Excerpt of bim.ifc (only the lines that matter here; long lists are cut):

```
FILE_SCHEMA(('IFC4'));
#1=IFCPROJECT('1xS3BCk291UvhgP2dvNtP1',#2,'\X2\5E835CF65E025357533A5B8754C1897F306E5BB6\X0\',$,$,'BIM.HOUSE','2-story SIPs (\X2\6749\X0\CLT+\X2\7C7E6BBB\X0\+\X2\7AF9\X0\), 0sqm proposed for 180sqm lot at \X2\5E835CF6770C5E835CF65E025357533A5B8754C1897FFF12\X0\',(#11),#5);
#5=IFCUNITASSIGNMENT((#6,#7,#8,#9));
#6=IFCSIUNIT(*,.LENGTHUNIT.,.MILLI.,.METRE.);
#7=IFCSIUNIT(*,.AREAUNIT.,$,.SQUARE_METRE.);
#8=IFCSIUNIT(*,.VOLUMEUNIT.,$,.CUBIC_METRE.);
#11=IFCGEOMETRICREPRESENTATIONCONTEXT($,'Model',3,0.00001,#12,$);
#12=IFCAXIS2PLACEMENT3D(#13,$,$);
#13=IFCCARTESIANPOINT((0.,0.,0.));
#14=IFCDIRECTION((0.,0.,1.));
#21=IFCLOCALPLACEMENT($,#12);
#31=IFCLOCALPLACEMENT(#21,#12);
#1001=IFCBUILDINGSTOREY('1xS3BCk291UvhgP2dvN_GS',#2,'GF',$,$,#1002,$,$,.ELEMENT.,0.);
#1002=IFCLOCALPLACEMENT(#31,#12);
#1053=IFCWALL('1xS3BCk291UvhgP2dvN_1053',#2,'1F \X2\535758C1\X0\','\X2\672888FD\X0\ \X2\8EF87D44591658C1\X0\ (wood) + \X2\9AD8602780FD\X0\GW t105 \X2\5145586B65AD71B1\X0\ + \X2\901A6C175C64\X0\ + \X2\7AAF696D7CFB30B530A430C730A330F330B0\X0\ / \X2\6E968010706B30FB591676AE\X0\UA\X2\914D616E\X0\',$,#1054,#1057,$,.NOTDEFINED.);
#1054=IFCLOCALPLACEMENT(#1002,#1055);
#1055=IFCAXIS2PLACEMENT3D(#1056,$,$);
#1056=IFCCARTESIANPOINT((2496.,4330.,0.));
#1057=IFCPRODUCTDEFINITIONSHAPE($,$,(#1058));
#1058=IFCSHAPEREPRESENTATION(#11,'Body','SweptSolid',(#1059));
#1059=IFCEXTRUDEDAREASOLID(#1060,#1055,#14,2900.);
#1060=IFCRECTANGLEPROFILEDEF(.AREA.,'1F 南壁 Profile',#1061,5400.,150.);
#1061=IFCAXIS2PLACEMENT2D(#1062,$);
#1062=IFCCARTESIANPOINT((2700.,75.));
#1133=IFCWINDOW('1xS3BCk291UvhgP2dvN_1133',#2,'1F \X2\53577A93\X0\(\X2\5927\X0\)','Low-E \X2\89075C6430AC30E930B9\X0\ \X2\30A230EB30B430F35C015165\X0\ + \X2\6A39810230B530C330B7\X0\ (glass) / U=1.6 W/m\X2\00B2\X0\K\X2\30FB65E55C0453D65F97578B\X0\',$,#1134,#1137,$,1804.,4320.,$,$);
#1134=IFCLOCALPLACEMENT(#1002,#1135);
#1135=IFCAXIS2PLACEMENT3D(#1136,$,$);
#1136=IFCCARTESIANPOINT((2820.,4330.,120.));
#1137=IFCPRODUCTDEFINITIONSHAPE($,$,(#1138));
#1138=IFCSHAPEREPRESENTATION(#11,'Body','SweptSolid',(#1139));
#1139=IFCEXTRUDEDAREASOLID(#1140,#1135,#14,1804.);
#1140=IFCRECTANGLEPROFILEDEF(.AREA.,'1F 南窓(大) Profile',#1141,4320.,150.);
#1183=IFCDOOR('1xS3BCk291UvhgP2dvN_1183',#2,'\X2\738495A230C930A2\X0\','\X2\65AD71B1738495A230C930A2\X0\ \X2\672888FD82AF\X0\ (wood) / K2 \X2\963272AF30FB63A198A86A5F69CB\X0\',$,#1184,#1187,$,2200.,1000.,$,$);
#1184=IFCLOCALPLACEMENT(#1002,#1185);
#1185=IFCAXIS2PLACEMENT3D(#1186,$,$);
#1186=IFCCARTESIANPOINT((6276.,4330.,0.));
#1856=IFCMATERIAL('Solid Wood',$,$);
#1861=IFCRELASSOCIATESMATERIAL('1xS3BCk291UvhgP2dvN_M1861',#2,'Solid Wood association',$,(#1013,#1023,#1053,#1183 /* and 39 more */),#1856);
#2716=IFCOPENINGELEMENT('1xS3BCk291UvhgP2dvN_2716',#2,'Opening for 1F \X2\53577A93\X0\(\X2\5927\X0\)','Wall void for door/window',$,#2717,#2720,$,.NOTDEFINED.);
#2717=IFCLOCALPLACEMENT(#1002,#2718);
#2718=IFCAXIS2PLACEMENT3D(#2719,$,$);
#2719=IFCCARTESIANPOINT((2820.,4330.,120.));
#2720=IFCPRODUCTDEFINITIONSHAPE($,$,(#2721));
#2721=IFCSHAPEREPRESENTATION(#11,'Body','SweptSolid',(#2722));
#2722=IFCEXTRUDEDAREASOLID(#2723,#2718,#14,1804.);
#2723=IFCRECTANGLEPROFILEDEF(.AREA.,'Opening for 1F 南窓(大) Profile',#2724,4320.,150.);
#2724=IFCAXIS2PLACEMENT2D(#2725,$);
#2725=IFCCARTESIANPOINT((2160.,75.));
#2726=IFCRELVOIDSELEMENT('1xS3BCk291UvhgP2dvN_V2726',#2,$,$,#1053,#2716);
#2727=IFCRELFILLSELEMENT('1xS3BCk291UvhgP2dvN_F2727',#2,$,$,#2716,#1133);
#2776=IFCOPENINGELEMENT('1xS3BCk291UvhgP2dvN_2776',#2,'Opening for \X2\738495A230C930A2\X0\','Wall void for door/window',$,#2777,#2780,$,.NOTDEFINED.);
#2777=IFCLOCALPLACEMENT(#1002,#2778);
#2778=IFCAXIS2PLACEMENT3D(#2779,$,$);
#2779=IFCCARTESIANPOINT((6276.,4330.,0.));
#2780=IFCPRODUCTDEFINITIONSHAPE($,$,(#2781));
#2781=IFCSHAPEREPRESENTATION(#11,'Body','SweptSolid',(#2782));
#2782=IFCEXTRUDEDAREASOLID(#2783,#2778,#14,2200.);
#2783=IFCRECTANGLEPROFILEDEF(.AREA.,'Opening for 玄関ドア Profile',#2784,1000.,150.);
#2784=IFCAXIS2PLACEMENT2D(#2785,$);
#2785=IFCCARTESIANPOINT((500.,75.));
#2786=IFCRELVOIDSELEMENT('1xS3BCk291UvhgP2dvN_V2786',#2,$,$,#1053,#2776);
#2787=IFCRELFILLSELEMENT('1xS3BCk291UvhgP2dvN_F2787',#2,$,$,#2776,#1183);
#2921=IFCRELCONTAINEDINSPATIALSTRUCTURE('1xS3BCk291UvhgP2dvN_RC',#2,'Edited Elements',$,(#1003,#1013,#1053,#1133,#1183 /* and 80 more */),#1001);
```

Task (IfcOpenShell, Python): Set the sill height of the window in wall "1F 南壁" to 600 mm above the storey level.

```python
import numpy as np
import ifcopenshell
import ifcopenshell.api.geometry
import ifcopenshell.geom
import ifcopenshell.util.element
import ifcopenshell.util.placement
import ifcopenshell.util.shape
import ifcopenshell.util.unit

model = ifcopenshell.open("bim.ifc")
unit_scale = ifcopenshell.util.unit.calculate_unit_scale(model)

window = model.by_id(1133)
opening = window.FillsVoids[0].RelatingOpeningElement
storey = ifcopenshell.util.element.get_container(window, ifc_class="IfcBuildingStorey")
level = ifcopenshell.util.placement.get_local_placement(storey.ObjectPlacement)[2, 3]

# The opening's origin need not be at the sill, so measure its lowest point.
shape = ifcopenshell.geom.create_shape(ifcopenshell.geom.settings(), opening)
bottom = ifcopenshell.util.shape.get_shape_bottom_elevation(shape, shape.geometry) / unit_scale
dz = level + 600.0 - bottom

shift = np.array([0.0, 0.0, dz])
# The window is not placed relative to its opening, so move both.
for product in (opening, window):
    matrix = ifcopenshell.util.placement.get_local_placement(product.ObjectPlacement)
    matrix[:3, 3] += shift
    ifcopenshell.api.geometry.edit_object_placement(model, product=product, matrix=matrix, is_si=False)

print(f"moved by {dz * unit_scale:+.3f} m")

model.write("bim-out.ifc")
```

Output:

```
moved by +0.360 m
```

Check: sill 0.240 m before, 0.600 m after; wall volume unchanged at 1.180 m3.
